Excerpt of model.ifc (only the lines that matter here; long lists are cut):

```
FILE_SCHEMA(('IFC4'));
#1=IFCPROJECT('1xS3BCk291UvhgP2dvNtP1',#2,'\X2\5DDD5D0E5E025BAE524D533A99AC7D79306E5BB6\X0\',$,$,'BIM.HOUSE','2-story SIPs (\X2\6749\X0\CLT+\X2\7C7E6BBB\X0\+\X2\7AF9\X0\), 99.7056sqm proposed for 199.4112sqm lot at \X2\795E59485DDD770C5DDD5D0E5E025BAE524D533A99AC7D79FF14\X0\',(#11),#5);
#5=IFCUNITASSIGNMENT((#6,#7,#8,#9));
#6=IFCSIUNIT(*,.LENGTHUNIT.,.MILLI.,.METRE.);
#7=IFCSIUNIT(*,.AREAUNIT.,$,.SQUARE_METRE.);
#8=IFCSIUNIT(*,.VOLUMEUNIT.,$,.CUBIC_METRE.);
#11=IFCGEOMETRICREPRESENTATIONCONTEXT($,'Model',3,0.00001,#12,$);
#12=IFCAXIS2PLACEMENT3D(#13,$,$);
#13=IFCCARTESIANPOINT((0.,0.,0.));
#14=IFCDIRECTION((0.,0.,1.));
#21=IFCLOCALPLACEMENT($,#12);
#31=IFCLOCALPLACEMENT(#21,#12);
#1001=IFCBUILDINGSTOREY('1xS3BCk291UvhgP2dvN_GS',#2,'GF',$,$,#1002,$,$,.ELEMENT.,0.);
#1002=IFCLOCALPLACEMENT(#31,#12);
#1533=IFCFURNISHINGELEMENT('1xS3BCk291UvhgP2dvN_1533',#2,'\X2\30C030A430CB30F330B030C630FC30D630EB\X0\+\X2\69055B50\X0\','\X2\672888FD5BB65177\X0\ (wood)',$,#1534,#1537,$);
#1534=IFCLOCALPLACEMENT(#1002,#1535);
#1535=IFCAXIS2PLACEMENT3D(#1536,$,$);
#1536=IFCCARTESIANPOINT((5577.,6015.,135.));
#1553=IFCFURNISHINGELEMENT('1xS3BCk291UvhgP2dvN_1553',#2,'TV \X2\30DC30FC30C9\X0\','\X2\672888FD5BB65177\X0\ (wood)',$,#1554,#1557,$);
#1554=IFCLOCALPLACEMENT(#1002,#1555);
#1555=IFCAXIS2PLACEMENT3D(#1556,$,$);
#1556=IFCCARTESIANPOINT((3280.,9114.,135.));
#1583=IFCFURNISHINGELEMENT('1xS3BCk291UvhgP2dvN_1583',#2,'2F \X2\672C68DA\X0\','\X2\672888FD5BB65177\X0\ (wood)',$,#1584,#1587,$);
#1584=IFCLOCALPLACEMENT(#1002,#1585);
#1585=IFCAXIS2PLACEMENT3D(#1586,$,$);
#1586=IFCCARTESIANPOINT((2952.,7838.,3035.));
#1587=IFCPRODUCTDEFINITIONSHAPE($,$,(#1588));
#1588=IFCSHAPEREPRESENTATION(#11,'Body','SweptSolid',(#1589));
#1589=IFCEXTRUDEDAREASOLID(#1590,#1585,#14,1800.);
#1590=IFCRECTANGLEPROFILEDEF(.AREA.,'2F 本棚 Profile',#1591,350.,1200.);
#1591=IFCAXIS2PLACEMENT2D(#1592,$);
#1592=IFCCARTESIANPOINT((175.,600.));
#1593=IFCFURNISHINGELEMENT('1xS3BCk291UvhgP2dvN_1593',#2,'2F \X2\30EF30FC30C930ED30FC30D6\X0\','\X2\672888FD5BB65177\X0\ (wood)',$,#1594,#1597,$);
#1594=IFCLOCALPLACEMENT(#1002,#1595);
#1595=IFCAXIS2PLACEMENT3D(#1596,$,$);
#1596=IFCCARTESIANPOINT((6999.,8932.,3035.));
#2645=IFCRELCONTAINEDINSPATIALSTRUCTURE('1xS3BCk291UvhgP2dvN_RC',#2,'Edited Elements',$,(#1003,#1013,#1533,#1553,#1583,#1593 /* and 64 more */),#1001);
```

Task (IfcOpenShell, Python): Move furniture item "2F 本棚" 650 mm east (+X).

```python
import ifcopenshell
import ifcopenshell.api.geometry
import ifcopenshell.util.placement

model = ifcopenshell.open("model.ifc")

item = model.by_guid("1xS3BCk291UvhgP2dvN_1583")
matrix = ifcopenshell.util.placement.get_local_placement(item.ObjectPlacement)
matrix[0, 3] += 650.0
ifcopenshell.api.geometry.edit_object_placement(model, product=item, matrix=matrix, is_si=False)

print(ifcopenshell.util.placement.get_local_placement(item.ObjectPlacement).round(3) + 0.0)

model.write("model_v2.ifc")
```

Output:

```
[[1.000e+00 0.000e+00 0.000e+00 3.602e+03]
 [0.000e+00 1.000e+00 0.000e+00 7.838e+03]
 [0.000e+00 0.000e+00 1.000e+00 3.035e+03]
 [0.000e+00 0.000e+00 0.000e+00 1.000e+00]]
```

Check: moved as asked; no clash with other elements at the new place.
